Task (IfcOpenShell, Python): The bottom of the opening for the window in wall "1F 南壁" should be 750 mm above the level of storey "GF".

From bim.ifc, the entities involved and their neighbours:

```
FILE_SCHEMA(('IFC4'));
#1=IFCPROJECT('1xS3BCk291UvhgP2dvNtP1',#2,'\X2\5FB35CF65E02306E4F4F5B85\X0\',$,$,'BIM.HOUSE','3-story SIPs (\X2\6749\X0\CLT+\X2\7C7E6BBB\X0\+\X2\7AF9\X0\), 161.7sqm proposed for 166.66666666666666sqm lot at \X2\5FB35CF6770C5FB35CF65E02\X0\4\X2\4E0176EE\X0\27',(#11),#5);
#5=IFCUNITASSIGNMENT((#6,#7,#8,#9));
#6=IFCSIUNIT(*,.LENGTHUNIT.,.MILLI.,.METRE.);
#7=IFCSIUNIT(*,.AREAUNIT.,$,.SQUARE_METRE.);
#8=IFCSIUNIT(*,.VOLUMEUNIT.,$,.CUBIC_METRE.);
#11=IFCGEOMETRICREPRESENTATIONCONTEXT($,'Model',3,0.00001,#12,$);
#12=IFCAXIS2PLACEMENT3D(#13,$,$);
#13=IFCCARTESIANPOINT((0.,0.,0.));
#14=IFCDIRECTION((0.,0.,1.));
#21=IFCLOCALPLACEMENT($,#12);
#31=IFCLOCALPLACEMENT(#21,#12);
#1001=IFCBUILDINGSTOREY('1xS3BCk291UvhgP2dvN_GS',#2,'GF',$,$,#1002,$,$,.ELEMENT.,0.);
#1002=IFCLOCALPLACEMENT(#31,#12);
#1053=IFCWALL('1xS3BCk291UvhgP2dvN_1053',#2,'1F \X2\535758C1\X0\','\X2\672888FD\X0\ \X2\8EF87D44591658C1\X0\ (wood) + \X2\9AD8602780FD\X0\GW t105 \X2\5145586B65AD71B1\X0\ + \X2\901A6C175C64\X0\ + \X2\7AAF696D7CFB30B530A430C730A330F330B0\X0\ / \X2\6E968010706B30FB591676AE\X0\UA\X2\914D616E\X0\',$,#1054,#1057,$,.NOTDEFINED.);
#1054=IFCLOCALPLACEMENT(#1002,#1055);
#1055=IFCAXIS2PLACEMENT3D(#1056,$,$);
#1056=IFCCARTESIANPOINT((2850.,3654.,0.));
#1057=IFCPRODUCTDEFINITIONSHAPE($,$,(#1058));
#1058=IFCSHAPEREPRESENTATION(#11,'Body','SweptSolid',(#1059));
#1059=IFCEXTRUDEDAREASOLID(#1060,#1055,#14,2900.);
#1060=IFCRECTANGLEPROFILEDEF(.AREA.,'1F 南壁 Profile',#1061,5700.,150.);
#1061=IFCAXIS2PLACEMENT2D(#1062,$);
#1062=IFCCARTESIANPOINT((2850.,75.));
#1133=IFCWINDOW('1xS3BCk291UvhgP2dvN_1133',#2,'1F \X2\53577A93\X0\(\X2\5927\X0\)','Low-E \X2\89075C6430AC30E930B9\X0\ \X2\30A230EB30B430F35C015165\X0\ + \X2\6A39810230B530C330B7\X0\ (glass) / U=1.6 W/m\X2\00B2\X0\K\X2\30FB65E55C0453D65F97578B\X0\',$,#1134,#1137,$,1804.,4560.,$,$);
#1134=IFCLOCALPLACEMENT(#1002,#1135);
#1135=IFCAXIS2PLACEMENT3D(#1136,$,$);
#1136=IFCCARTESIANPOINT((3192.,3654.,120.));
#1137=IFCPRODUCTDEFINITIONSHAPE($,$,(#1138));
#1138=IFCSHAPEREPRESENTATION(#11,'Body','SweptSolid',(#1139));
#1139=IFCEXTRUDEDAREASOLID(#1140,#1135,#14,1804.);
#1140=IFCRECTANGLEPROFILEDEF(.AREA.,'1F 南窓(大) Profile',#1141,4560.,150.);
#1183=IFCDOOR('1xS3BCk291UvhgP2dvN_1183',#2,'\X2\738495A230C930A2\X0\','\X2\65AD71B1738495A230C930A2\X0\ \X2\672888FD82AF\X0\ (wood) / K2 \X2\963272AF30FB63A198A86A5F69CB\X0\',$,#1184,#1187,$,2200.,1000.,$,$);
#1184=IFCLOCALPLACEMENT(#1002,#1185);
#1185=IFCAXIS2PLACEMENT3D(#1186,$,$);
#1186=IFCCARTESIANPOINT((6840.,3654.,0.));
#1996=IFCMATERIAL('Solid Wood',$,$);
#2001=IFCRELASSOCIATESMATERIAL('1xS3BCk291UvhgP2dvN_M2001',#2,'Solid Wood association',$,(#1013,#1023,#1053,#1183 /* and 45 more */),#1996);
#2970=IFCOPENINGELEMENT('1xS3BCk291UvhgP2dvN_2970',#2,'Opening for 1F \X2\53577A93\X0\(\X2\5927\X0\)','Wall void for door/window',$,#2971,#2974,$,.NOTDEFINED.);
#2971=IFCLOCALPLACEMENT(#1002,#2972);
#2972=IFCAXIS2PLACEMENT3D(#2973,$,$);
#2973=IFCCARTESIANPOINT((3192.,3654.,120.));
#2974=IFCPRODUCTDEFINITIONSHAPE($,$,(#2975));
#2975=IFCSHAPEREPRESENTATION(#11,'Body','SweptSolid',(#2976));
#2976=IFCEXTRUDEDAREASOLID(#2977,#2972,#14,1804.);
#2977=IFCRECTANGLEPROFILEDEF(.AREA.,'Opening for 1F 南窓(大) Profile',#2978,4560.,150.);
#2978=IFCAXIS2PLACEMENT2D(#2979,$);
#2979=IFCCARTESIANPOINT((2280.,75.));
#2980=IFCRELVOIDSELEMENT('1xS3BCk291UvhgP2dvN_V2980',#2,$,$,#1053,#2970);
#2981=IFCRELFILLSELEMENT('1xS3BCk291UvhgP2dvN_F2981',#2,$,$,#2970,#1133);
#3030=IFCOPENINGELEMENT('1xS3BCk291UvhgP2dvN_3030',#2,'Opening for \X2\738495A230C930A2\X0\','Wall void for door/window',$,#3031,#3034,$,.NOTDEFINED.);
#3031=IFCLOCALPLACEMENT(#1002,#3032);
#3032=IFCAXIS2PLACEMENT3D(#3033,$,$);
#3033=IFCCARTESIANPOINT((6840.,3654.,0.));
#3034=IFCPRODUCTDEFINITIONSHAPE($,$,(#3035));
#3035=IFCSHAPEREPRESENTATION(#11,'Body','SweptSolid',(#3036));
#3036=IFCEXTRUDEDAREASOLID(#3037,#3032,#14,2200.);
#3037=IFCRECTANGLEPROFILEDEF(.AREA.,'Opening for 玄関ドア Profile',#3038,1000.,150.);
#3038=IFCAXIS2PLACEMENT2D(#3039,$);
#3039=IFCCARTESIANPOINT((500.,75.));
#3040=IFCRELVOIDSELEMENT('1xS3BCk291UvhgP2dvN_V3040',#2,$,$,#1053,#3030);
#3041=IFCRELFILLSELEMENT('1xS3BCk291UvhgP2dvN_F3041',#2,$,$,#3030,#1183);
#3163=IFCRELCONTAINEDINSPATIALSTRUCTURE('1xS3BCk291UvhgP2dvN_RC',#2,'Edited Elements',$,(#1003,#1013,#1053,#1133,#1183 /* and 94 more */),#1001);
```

```python
import numpy as np
import ifcopenshell
import ifcopenshell.api.geometry
import ifcopenshell.geom
import ifcopenshell.util.element
import ifcopenshell.util.placement
import ifcopenshell.util.shape
import ifcopenshell.util.unit

model = ifcopenshell.open("bim.ifc")
unit_scale = ifcopenshell.util.unit.calculate_unit_scale(model)

window = model.by_guid("1xS3BCk291UvhgP2dvN_1133")
opening = window.FillsVoids[0].RelatingOpeningElement
storey = ifcopenshell.util.element.get_container(window, ifc_class="IfcBuildingStorey")
level = ifcopenshell.util.placement.get_local_placement(storey.ObjectPlacement)[2, 3]

# The opening's origin need not be at the sill, so measure its lowest point.
shape = ifcopenshell.geom.create_shape(ifcopenshell.geom.settings(), opening)
bottom = ifcopenshell.util.shape.get_shape_bottom_elevation(shape, shape.geometry) / unit_scale
dz = level + 0.75 / unit_scale - bottom

shift = np.array([0.0, 0.0, dz])
# The window is not placed relative to its opening, so move both.
for product in (opening, window):
    matrix = ifcopenshell.util.placement.get_local_placement(product.ObjectPlacement)
    matrix[:3, 3] += shift
    ifcopenshell.api.geometry.edit_object_placement(model, product=product, matrix=matrix, is_si=False)

print(f"moved by {dz * unit_scale:+.3f} m")

model.write("bim_v2.ifc")
```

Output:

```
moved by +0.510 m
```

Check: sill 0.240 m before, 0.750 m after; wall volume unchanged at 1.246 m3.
